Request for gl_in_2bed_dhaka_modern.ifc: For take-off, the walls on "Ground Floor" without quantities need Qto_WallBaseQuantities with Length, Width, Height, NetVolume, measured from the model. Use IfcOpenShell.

First a look at what the model holds.

```python
import ifcopenshell
import ifcopenshell.util.element
import ifcopenshell.util.unit

model = ifcopenshell.open("gl_in_2bed_dhaka_modern.ifc")
print(model.schema)
for unit_type in ("LENGTHUNIT", "AREAUNIT", "VOLUMEUNIT"):
    print(unit_type, ifcopenshell.util.unit.calculate_unit_scale(model, unit_type))
storey = next(s for s in model.by_type("IfcBuildingStorey") if s.Name == "Ground Floor")
walls = [e for e in ifcopenshell.util.element.get_decomposition(storey) if e.is_a("IfcWall")]
for e in sorted(walls, key=lambda e: e.id()):
    print(e.id(), e.is_a(), e.Name, list(ifcopenshell.util.element.get_psets(e, qtos_only=True)), sep=" | ")
```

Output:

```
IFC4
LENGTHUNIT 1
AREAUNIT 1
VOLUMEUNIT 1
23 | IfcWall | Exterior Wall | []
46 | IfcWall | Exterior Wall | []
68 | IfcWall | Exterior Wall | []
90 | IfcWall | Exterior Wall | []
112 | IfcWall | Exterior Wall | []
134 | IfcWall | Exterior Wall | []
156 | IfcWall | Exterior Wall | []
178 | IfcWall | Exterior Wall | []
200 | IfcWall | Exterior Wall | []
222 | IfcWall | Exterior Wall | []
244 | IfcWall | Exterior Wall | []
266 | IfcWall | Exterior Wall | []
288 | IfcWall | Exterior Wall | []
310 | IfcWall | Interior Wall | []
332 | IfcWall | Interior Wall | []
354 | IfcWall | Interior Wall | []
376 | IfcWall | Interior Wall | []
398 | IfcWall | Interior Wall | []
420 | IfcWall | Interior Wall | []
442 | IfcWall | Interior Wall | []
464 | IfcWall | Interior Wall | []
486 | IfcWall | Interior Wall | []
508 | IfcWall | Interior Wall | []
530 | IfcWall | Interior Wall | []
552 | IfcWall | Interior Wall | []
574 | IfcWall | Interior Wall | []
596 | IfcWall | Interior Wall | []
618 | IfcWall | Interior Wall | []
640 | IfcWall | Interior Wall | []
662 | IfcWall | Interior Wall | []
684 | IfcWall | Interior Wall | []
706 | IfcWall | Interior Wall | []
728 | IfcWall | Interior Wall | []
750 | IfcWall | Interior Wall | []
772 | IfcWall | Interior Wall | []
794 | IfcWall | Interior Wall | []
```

```python
import ifcopenshell
import ifcopenshell.api.pset
import ifcopenshell.geom
import ifcopenshell.util.element
import ifcopenshell.util.shape
import ifcopenshell.util.unit

model = ifcopenshell.open("gl_in_2bed_dhaka_modern.ifc")
unit_scale = ifcopenshell.util.unit.calculate_unit_scale(model)
volume_scale = ifcopenshell.util.unit.calculate_unit_scale(model, "VOLUMEUNIT")
settings = ifcopenshell.geom.settings()

storey = next(s for s in model.by_type("IfcBuildingStorey") if s.Name == "Ground Floor")
walls = [e for e in ifcopenshell.util.element.get_decomposition(storey) if e.is_a("IfcWall")]

for e in sorted(walls, key=lambda e: e.id()):
    if ifcopenshell.util.element.get_psets(e, qtos_only=True, should_inherit=False):
        continue
    # Geometry comes back in metres, in the element's own axes.
    shape = ifcopenshell.geom.create_shape(settings, e)
    values = {
        "Length": ifcopenshell.util.shape.get_x(shape.geometry) / unit_scale,
        "Width": ifcopenshell.util.shape.get_y(shape.geometry) / unit_scale,
        "Height": ifcopenshell.util.shape.get_z(shape.geometry) / unit_scale,
        "NetVolume": ifcopenshell.util.shape.get_volume(shape.geometry) / volume_scale,
    }
    qto = ifcopenshell.api.pset.add_qto(model, product=e, name="Qto_WallBaseQuantities")
    ifcopenshell.api.pset.edit_qto(model, qto=qto, properties=values)
    print(e.id(), {k: round(v, 3) for k, v in values.items()})

model.write("gl_in_2bed_dhaka_modern_updated.ifc")
```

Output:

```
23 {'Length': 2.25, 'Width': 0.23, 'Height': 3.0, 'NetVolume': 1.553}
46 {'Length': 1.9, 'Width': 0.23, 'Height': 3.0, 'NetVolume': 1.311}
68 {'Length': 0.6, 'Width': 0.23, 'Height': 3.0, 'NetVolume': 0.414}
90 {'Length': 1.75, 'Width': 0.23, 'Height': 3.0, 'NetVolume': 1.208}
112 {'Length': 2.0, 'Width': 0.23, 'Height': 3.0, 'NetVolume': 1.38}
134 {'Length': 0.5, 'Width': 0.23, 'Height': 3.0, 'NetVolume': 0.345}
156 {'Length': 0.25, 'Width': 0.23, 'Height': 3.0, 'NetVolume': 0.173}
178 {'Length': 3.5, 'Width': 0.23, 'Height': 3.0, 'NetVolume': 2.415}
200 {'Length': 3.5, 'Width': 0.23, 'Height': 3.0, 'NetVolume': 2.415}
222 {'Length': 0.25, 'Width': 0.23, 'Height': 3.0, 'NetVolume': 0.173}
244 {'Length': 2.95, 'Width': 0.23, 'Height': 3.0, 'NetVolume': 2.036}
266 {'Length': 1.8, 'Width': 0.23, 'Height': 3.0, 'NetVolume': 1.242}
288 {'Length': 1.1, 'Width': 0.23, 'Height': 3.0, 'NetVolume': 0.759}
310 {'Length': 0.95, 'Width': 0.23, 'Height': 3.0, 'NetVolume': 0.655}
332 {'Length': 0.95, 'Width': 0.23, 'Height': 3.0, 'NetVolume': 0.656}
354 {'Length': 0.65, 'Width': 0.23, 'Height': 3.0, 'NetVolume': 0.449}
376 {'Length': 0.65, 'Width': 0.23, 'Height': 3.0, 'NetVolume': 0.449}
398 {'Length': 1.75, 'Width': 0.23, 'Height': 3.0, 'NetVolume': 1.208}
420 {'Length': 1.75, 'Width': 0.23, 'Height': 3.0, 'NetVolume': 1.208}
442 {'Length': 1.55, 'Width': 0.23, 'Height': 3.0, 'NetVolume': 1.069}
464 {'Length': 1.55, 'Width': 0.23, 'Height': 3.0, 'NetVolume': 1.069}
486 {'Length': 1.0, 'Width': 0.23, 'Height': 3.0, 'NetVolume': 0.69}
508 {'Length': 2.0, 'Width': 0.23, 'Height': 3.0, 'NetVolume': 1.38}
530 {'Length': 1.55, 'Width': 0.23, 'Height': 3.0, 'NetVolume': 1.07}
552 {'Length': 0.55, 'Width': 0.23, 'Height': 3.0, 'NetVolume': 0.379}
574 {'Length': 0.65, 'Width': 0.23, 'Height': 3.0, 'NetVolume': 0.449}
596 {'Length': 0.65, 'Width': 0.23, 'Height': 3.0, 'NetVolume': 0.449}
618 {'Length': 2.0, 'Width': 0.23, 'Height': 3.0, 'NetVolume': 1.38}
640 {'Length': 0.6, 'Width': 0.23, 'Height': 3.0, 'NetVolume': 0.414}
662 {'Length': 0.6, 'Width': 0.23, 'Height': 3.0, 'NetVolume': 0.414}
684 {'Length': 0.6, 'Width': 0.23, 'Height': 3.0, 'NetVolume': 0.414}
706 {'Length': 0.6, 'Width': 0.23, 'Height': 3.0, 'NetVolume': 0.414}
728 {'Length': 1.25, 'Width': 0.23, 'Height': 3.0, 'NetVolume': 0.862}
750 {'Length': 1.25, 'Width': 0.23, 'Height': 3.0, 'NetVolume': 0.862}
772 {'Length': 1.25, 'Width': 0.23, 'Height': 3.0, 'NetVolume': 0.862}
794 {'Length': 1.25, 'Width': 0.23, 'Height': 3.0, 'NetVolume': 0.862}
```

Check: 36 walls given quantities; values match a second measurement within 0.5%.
